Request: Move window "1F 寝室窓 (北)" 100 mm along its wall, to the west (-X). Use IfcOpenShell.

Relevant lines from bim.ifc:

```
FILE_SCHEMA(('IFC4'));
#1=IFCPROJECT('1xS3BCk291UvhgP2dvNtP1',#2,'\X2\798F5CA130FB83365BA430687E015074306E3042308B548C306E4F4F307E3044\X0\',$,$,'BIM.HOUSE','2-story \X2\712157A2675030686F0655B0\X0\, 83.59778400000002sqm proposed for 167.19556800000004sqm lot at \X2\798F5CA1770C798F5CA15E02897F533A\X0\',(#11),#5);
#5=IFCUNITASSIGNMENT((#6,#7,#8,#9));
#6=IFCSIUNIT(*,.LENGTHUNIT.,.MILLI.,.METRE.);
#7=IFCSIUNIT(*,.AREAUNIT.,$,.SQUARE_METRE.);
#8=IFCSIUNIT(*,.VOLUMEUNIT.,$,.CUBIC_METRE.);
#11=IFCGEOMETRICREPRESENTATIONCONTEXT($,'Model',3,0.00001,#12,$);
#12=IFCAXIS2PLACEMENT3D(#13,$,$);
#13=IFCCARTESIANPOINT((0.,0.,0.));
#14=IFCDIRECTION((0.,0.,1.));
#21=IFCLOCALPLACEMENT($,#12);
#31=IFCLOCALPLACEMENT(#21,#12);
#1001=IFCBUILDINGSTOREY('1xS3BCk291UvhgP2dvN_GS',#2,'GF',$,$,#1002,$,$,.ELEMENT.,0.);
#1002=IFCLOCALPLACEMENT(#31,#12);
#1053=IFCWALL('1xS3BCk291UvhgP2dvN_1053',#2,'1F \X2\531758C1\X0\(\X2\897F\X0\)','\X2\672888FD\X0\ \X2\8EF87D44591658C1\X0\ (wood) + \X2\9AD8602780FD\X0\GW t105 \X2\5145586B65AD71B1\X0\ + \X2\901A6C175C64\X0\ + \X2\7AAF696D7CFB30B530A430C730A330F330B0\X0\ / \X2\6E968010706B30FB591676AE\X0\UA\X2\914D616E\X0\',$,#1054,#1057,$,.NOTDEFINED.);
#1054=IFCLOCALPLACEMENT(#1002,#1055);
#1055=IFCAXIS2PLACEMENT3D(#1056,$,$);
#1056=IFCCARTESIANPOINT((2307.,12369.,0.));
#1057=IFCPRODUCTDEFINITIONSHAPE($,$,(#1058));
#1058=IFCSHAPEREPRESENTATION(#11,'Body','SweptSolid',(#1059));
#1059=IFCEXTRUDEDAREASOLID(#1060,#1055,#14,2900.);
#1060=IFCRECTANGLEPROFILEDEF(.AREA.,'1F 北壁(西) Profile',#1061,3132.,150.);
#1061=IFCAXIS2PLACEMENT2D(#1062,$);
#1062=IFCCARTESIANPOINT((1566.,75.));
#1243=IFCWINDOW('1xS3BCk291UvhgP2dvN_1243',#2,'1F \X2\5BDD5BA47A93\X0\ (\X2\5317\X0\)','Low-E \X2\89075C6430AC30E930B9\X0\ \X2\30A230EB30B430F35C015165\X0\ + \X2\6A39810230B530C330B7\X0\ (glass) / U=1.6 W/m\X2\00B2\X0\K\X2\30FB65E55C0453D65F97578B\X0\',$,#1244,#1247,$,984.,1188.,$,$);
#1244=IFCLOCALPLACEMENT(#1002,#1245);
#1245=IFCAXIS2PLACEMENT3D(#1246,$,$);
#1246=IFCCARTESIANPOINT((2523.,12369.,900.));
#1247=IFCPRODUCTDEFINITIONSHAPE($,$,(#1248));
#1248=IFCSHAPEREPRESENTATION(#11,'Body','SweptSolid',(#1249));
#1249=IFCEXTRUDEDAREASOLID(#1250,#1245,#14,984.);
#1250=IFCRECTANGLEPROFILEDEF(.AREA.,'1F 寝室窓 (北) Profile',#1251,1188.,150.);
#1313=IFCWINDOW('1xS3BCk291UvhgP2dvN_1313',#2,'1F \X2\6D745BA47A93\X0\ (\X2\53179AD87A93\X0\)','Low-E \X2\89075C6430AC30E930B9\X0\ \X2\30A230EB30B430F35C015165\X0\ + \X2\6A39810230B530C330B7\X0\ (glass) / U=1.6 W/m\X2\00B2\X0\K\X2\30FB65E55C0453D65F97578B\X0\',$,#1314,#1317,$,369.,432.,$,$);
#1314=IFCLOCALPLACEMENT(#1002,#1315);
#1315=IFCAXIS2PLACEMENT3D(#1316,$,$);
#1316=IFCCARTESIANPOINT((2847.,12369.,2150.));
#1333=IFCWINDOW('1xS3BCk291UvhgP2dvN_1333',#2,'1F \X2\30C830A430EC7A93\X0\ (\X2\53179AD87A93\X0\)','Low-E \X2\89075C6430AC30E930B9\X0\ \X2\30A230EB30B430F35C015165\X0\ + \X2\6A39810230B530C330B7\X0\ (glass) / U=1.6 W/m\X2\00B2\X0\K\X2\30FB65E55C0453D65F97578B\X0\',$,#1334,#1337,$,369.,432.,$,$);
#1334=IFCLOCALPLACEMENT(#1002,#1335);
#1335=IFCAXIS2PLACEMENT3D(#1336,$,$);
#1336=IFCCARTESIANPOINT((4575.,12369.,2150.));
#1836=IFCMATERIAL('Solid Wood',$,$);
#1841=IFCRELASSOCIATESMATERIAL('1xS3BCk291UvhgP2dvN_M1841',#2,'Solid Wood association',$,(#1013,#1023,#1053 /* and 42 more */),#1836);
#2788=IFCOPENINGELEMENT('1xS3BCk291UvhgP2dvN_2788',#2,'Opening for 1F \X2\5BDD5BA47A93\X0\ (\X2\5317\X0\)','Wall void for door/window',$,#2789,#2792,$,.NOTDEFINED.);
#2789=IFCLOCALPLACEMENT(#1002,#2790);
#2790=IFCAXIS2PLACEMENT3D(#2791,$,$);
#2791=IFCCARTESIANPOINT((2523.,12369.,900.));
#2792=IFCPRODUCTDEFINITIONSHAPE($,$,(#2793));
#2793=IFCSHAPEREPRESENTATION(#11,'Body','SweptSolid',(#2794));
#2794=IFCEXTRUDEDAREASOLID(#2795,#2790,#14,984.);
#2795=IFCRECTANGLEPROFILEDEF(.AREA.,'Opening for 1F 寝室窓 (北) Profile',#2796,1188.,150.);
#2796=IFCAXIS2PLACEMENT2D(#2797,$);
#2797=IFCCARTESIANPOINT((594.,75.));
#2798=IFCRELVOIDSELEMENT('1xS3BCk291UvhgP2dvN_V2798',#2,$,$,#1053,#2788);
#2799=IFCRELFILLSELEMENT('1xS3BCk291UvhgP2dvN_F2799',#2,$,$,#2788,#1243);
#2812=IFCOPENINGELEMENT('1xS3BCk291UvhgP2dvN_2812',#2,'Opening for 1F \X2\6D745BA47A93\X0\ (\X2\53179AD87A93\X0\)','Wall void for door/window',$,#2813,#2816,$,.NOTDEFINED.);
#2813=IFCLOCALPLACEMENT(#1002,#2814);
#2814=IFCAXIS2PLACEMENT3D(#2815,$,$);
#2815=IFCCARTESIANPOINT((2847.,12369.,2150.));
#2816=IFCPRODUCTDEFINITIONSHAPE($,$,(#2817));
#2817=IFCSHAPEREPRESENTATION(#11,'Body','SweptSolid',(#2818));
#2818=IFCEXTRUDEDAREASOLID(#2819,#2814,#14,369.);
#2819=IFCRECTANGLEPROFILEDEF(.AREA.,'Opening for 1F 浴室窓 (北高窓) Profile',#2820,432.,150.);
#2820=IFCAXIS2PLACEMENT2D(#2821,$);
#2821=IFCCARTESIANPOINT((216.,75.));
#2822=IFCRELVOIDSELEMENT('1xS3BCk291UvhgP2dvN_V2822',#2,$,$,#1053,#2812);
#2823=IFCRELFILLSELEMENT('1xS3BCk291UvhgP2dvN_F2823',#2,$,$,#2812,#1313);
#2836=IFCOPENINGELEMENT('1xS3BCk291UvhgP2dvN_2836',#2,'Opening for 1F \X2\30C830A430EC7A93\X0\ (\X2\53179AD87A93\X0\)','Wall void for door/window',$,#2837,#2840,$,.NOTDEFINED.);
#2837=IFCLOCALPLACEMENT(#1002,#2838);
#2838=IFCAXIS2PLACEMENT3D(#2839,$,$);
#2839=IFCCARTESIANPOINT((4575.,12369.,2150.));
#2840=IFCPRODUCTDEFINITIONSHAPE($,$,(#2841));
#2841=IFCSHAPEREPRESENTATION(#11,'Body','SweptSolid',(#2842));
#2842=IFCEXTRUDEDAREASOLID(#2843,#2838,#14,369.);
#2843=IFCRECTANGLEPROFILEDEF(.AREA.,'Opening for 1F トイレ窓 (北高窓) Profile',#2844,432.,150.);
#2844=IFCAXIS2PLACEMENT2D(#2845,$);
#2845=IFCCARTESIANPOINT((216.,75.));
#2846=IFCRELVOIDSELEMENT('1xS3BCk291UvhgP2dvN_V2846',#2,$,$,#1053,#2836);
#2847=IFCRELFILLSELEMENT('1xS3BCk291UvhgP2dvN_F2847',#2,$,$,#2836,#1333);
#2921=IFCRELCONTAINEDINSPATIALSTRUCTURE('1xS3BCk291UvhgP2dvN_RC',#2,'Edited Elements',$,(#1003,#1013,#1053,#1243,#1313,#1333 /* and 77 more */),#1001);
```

```python
import ifcopenshell
import ifcopenshell.api.geometry
import ifcopenshell.util.placement

model = ifcopenshell.open("bim.ifc")

window = model.by_guid("1xS3BCk291UvhgP2dvN_1243")
opening = window.FillsVoids[0].RelatingOpeningElement
wall = opening.VoidsElements[0].RelatingBuildingElement

wall_matrix = ifcopenshell.util.placement.get_local_placement(wall.ObjectPlacement)
shift = wall_matrix[:3, 0] * -100.0
before = ifcopenshell.util.placement.get_local_placement(window.ObjectPlacement)[:3, 3].copy()

# The window is not placed relative to its opening, so move both.
for product in (opening, window):
    matrix = ifcopenshell.util.placement.get_local_placement(product.ObjectPlacement)
    matrix[:3, 3] += shift
    ifcopenshell.api.geometry.edit_object_placement(model, product=product, matrix=matrix, is_si=False)

after = ifcopenshell.util.placement.get_local_placement(window.ObjectPlacement)[:3, 3]
print("window moved by", (after - before).round(3) + 0.0)

model.write("bim_updated.ifc")
```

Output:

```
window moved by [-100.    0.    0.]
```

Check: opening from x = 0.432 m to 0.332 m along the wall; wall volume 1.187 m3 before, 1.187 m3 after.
